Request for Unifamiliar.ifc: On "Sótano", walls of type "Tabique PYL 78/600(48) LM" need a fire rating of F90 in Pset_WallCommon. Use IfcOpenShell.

First a look at what the model holds.

```python
import ifcopenshell
import ifcopenshell.util.element

model = ifcopenshell.open("Unifamiliar.ifc")
print(model.schema)
storey = next(s for s in model.by_type("IfcBuildingStorey") if s.Name == "Sótano")
walls = [e for e in ifcopenshell.util.element.get_decomposition(storey) if e.is_a("IfcWall")]
seen = {}
for e in walls:
    element_type = ifcopenshell.util.element.get_type(e)
    key = (element_type.Name if element_type != e and element_type else None, ifcopenshell.util.element.get_pset(e, "Pset_WallCommon", "FireRating"))
    seen[key] = seen.get(key, 0) + 1
for (name, value), count in sorted(seen.items(), key=str):
    print(count, "x", name, "|", value)
```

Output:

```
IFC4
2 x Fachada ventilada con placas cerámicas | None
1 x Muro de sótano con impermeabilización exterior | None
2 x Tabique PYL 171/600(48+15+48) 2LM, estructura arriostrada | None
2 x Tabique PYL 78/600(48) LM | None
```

```python
import ifcopenshell
import ifcopenshell.api.pset
import ifcopenshell.util.element

model = ifcopenshell.open("Unifamiliar.ifc")

storey = next(s for s in model.by_type("IfcBuildingStorey") if s.Name == "Sótano")
walls = [e for e in ifcopenshell.util.element.get_decomposition(storey) if e.is_a("IfcWall")]

count = 0
for e in walls:
    element_type = ifcopenshell.util.element.get_type(e)
    if element_type in (None, e) or element_type.Name != "Tabique PYL 78/600(48) LM":
        continue
    # add_pset returns the element's existing set when there is one.
    pset = ifcopenshell.api.pset.add_pset(model, product=e, name="Pset_WallCommon")
    ifcopenshell.api.pset.edit_pset(model, pset=pset, properties={"FireRating": "F90"})
    count += 1

print(count, "walls updated")

model.write("Unifamiliar_rev.ifc")
```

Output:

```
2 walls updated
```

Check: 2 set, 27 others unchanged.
